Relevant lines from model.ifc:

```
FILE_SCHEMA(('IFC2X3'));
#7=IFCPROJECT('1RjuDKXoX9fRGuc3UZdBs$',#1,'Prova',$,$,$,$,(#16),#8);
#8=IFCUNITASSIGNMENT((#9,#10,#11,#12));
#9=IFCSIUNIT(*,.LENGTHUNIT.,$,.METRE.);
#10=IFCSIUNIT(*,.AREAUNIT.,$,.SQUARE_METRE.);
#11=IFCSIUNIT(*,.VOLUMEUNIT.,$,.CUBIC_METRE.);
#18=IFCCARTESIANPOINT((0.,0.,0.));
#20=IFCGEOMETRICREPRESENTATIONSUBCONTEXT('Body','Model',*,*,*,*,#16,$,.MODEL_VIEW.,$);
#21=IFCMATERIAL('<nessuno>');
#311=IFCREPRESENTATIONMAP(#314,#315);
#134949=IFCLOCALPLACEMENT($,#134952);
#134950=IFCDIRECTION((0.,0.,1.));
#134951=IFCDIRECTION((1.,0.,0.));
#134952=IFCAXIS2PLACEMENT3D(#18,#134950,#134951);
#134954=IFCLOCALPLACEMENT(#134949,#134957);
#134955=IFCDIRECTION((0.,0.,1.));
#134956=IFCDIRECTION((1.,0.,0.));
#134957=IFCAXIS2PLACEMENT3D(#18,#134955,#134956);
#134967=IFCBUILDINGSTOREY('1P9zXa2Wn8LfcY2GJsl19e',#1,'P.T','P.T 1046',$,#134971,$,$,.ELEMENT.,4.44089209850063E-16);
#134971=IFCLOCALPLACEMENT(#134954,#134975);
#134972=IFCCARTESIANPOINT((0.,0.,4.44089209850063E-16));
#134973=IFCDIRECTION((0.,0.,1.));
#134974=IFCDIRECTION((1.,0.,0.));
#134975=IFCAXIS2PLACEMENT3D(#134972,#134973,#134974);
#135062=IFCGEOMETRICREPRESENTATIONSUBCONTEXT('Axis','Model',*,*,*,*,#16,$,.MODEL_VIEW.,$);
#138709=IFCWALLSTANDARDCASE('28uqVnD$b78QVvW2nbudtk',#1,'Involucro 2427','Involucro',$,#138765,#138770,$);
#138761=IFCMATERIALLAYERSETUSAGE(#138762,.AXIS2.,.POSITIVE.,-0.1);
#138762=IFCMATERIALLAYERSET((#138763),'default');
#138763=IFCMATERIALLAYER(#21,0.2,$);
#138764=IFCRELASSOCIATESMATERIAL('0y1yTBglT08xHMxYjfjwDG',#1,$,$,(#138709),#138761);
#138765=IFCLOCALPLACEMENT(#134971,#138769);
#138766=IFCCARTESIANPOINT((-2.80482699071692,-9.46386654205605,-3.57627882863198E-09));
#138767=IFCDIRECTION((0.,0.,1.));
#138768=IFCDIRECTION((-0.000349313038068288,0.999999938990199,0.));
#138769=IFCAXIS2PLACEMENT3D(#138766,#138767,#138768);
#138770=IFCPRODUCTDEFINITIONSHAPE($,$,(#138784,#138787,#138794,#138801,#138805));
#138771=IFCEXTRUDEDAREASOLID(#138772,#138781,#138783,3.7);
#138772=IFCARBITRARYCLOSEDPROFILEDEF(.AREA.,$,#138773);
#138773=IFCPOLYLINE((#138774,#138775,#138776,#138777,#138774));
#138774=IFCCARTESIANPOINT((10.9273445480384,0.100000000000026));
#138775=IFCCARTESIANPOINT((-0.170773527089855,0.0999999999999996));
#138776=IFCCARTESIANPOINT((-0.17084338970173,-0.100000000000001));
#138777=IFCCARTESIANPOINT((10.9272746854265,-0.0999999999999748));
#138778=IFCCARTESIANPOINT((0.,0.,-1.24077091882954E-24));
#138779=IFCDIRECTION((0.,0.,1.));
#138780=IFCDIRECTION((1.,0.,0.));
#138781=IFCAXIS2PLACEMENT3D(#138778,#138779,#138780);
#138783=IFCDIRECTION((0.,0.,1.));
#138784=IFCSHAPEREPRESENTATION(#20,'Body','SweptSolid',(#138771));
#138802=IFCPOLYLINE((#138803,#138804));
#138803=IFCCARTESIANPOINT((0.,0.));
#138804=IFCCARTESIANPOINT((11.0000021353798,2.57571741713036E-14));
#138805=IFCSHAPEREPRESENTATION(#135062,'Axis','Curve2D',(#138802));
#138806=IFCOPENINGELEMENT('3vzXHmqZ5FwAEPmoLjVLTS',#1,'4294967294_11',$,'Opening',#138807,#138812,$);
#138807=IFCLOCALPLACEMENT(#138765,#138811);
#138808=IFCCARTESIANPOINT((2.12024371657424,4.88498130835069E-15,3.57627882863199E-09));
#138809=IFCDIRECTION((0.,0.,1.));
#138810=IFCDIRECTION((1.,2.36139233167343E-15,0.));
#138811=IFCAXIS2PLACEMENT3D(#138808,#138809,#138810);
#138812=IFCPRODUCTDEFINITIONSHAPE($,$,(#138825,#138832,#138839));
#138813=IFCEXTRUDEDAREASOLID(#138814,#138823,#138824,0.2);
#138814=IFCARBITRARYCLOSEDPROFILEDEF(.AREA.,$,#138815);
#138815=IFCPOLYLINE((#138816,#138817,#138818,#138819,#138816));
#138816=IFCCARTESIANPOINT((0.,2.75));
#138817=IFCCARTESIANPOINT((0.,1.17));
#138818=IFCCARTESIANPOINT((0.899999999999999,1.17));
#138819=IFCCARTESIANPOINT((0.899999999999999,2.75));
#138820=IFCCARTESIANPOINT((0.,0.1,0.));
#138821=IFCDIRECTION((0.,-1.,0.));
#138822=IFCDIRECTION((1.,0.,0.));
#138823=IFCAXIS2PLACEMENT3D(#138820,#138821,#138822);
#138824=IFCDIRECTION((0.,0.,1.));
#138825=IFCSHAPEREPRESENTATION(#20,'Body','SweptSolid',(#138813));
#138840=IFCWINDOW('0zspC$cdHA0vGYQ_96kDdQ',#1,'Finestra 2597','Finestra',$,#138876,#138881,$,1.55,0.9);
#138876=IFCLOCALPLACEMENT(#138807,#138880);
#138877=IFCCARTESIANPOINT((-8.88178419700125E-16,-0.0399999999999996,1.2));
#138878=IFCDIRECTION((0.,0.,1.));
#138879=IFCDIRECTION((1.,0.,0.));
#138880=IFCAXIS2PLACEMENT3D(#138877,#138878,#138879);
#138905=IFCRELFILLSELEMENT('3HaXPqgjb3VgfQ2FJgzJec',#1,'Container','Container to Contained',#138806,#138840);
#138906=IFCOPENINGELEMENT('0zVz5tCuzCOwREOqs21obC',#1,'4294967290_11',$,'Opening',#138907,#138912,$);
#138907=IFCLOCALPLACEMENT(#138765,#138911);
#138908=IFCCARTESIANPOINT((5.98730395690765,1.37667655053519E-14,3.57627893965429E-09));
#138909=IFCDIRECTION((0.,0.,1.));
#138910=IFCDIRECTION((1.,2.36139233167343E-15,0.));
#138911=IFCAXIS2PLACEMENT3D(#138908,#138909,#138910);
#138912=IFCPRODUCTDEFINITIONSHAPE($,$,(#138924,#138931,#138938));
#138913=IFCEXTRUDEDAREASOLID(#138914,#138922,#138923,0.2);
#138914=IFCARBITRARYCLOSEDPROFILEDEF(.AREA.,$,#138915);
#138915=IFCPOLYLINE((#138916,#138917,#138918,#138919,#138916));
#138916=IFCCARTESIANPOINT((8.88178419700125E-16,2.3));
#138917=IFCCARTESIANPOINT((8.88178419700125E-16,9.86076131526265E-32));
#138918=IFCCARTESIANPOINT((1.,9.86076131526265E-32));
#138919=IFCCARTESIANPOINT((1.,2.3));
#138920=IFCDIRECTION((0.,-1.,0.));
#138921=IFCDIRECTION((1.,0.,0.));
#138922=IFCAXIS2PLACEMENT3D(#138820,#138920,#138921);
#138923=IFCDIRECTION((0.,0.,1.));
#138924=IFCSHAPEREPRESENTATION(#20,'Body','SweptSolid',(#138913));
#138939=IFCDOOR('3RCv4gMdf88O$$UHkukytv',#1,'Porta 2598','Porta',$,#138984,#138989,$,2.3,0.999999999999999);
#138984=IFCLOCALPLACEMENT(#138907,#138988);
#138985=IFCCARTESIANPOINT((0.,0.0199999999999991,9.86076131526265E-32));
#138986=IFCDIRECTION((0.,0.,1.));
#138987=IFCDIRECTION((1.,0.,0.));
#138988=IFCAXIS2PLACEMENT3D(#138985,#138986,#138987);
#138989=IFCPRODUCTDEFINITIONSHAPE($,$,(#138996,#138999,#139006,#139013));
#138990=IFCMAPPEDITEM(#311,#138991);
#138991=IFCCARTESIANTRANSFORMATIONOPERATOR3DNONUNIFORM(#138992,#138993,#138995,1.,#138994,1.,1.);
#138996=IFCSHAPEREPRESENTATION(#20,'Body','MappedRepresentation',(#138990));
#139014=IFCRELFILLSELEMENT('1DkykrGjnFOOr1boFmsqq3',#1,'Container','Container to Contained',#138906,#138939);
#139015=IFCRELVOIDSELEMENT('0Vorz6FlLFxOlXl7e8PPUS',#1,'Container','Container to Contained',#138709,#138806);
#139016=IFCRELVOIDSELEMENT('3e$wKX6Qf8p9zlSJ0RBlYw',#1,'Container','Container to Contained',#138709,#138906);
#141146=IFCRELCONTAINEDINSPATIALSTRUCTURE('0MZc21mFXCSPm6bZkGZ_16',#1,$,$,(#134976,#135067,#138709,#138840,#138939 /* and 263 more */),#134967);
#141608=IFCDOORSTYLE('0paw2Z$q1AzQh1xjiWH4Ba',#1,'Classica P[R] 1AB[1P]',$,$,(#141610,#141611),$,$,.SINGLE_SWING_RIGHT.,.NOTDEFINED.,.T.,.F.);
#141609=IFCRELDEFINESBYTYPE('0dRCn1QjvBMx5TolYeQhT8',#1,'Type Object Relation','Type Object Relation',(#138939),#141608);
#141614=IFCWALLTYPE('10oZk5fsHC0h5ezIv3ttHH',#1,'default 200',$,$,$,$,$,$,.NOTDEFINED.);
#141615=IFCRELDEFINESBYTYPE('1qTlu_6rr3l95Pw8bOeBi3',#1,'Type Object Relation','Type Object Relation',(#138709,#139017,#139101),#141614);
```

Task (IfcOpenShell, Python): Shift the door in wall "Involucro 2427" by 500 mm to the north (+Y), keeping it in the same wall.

```python
import ifcopenshell
import ifcopenshell.api.geometry
import ifcopenshell.util.placement
import ifcopenshell.util.unit

model = ifcopenshell.open("model.ifc")
unit_scale = ifcopenshell.util.unit.calculate_unit_scale(model)

door = model.by_id(138939)
opening = door.FillsVoids[0].RelatingOpeningElement
wall = opening.VoidsElements[0].RelatingBuildingElement

wall_matrix = ifcopenshell.util.placement.get_local_placement(wall.ObjectPlacement)
shift = wall_matrix[:3, 0] * 0.5 / unit_scale
before = ifcopenshell.util.placement.get_local_placement(door.ObjectPlacement)[:3, 3].copy()

# The door is placed relative to its opening, so it follows when the opening moves.
matrix = ifcopenshell.util.placement.get_local_placement(opening.ObjectPlacement)
matrix[:3, 3] += shift
ifcopenshell.api.geometry.edit_object_placement(
    model, product=opening, matrix=matrix, is_si=False, should_transform_children=True
)

after = ifcopenshell.util.placement.get_local_placement(door.ObjectPlacement)[:3, 3]
print("door moved by", (after - before).round(3) + 0.0)

model.write("model_rev.ifc")
```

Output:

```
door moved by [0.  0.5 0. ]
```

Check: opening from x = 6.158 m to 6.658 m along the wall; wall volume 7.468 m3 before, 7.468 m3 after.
